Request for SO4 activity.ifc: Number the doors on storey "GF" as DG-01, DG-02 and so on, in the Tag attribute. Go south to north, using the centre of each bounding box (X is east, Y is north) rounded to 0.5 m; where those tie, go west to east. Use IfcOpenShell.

First a look at what the model holds.

```python
import ifcopenshell
import ifcopenshell.util.element
import ifcopenshell.util.placement

model = ifcopenshell.open("SO4 activity.ifc")
print(model.schema)
storey = next(s for s in model.by_type("IfcBuildingStorey") if s.Name == "GF")
doors = [e for e in ifcopenshell.util.element.get_decomposition(storey) if e.is_a("IfcDoor")]
for e in sorted(doors, key=lambda e: e.id()):
    origin = ifcopenshell.util.placement.get_local_placement(e.ObjectPlacement)[:3, 3]
    print(e.id(), e.Tag, e.Name, origin.round(2) + 0.0, sep=" | ")
```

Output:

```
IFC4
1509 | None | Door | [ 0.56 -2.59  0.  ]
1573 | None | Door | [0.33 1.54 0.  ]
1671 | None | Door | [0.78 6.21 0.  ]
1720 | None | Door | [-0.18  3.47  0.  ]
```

```python
import ifcopenshell
import ifcopenshell.geom
import ifcopenshell.util.element
import ifcopenshell.util.shape

model = ifcopenshell.open("SO4 activity.ifc")
settings = ifcopenshell.geom.settings()
settings.set("use-world-coords", True)


def centre(element):
    shape = ifcopenshell.geom.create_shape(settings, element)
    return ifcopenshell.util.shape.get_bbox_centroid(shape.geometry)


storey = next(s for s in model.by_type("IfcBuildingStorey") if s.Name == "GF")
doors = [e for e in ifcopenshell.util.element.get_decomposition(storey) if e.is_a("IfcDoor")]

# Insertion points can sit at a corner or the storey origin, so sort by the geometry (in metres).
centres = {e: centre(e) for e in doors}
doors.sort(key=lambda e: (round(centres[e][1] / 0.5), centres[e][0]))

for i, e in enumerate(doors, start=1):
    number = f"DG-{i:02d}"
    e.Tag = number
    print(e.id(), number)

model.write("SO4 activity_rev.ifc")
```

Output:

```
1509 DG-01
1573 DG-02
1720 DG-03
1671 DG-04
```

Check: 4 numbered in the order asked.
